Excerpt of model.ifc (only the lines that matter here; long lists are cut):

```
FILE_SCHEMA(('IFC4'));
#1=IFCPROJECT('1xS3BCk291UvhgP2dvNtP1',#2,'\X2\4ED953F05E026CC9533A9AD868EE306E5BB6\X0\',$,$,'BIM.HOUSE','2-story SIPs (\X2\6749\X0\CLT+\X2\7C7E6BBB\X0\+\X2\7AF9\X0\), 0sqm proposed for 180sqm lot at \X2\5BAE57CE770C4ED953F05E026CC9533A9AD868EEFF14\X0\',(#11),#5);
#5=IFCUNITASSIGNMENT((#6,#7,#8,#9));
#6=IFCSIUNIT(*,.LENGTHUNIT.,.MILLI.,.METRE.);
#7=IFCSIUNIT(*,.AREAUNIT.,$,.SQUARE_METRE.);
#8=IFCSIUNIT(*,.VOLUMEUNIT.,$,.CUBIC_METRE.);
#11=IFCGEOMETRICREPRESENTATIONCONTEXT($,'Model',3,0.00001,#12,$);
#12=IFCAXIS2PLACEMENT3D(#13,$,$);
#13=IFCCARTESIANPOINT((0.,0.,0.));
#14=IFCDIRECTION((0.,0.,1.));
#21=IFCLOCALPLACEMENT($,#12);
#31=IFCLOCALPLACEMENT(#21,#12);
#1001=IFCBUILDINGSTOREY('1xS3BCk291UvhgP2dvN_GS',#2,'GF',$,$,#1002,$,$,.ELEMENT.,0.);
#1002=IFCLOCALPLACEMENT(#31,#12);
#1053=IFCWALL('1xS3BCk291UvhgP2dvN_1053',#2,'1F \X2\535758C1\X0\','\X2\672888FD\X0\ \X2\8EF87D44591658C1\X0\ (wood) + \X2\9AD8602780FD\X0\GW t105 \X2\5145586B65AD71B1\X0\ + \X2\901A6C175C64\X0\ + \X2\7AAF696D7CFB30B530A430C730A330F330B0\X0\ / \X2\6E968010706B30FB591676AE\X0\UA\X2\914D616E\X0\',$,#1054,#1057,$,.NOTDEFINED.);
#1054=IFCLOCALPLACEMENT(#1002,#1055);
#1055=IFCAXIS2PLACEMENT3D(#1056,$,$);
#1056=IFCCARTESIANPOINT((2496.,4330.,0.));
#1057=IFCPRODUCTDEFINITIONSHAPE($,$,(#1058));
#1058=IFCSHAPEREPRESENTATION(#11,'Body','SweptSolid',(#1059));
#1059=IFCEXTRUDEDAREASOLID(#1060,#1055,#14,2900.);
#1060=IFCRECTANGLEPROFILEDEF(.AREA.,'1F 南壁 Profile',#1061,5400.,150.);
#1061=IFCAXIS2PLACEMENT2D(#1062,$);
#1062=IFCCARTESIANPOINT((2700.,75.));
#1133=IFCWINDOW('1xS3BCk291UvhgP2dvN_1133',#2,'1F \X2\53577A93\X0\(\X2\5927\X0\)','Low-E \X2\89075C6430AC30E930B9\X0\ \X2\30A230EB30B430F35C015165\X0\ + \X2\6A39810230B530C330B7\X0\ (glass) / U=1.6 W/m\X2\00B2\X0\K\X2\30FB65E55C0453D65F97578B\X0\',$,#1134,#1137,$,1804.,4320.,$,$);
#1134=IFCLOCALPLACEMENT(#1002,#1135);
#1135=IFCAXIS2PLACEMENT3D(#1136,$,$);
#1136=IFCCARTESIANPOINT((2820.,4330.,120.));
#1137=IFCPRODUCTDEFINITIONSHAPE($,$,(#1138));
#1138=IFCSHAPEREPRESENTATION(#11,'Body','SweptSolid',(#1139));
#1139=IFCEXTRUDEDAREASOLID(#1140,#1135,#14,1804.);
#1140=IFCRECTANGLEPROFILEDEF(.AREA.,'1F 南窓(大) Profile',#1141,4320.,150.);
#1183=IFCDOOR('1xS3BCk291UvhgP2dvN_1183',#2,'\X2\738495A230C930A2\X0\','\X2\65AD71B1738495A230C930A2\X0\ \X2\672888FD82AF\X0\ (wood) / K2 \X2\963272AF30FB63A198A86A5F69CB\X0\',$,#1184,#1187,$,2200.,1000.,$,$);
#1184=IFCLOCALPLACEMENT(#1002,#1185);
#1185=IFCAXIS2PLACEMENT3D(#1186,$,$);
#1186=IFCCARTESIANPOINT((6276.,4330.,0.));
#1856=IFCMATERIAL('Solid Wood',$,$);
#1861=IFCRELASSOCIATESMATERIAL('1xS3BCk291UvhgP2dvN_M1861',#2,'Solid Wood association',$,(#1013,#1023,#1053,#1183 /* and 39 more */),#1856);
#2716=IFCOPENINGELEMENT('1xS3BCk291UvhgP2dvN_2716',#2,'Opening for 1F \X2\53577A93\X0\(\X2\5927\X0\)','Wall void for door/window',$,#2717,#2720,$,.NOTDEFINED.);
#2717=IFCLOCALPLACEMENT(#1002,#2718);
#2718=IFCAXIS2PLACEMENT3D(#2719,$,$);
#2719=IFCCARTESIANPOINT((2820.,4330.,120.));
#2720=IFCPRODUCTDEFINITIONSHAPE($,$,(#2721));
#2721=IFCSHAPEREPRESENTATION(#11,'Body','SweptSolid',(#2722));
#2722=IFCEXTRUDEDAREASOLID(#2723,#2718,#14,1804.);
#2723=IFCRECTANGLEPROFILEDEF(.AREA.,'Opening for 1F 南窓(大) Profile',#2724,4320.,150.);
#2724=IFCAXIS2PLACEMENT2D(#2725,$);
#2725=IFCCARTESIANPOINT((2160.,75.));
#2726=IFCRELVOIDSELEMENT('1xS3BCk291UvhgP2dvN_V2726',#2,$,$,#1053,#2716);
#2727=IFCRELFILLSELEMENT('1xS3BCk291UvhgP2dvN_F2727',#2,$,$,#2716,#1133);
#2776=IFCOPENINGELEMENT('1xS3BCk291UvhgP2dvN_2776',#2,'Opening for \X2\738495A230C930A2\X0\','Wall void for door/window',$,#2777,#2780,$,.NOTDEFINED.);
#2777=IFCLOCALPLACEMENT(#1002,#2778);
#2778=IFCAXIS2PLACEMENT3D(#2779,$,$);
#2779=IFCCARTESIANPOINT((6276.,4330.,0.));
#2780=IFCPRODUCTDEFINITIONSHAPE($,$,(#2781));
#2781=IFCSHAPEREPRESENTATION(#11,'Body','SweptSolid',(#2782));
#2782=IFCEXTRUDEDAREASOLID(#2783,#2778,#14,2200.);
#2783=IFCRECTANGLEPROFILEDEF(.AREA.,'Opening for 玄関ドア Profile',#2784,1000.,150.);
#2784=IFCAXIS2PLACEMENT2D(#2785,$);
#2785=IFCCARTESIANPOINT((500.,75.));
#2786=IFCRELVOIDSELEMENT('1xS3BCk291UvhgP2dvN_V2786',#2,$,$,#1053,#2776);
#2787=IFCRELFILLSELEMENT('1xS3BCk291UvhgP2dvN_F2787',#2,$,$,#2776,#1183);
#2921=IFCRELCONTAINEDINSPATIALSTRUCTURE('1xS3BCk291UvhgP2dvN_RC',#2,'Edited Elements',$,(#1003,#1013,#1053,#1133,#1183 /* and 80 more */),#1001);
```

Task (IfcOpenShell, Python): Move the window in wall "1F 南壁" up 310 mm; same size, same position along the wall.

```python
import numpy as np
import ifcopenshell
import ifcopenshell.api.geometry
import ifcopenshell.util.placement
import ifcopenshell.util.unit

model = ifcopenshell.open("model.ifc")
unit_scale = ifcopenshell.util.unit.calculate_unit_scale(model)

window = model.by_guid("1xS3BCk291UvhgP2dvN_1133")
opening = window.FillsVoids[0].RelatingOpeningElement
dz = 310.0

shift = np.array([0.0, 0.0, dz])
# The window is not placed relative to its opening, so move both.
for product in (opening, window):
    matrix = ifcopenshell.util.placement.get_local_placement(product.ObjectPlacement)
    matrix[:3, 3] += shift
    ifcopenshell.api.geometry.edit_object_placement(model, product=product, matrix=matrix, is_si=False)

print(f"moved by {dz * unit_scale:+.3f} m")

model.write("model-out.ifc")
```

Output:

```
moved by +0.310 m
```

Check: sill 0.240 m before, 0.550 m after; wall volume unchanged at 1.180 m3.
